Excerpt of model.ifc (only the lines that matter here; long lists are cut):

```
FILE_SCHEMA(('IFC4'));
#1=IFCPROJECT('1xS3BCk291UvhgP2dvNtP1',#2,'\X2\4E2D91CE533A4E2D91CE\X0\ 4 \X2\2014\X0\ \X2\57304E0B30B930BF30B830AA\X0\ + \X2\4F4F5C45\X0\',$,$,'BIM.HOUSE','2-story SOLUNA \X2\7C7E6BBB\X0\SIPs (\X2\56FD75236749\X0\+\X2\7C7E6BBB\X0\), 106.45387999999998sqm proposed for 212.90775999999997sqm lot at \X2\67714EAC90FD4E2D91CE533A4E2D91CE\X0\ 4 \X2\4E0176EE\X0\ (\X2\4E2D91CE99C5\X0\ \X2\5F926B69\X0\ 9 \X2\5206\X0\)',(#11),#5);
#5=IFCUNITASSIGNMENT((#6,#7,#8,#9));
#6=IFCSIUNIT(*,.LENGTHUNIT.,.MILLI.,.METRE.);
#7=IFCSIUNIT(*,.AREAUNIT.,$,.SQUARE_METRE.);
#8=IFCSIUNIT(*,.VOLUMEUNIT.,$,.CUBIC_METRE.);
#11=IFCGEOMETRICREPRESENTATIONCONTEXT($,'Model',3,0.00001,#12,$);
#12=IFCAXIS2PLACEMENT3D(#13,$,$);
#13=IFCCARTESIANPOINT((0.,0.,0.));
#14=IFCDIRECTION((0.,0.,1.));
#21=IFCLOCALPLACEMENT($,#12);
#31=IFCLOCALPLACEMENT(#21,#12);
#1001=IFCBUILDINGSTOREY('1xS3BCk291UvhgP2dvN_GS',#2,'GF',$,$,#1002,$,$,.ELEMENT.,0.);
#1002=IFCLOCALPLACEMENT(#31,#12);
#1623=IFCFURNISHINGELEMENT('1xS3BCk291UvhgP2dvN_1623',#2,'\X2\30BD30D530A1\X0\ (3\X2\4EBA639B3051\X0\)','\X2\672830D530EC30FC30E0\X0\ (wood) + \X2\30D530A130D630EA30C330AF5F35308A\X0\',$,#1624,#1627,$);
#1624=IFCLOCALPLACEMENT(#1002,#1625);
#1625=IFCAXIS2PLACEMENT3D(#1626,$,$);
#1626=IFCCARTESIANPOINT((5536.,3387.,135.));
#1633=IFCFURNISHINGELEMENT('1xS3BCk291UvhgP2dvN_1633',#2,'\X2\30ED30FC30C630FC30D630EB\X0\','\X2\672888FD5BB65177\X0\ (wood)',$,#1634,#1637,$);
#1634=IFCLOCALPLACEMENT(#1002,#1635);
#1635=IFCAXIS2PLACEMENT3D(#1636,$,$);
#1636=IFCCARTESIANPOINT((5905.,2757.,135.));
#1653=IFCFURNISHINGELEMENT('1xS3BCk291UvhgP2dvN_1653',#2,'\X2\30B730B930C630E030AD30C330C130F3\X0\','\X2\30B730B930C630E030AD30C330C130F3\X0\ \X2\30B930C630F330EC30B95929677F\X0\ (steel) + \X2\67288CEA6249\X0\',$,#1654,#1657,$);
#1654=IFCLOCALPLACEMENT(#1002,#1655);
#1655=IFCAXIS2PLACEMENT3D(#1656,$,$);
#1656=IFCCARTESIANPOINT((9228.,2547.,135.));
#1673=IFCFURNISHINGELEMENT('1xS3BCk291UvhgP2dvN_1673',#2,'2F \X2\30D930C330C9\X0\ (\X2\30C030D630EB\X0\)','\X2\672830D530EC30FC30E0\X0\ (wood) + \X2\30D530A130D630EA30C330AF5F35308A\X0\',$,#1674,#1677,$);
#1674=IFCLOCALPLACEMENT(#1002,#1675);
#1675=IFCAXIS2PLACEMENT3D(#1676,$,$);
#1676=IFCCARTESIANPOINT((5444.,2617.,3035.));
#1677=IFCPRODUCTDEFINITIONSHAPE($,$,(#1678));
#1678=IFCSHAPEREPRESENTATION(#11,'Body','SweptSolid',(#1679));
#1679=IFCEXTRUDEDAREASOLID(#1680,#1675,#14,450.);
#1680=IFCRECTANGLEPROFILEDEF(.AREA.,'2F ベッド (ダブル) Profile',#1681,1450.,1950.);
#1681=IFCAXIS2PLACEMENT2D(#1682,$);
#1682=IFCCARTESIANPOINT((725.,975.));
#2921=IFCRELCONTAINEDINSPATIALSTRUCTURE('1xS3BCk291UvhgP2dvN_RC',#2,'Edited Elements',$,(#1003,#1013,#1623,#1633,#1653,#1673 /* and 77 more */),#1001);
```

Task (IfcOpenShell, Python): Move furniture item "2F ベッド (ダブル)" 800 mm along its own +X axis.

```python
import ifcopenshell
import ifcopenshell.api.geometry
import ifcopenshell.util.placement

model = ifcopenshell.open("model.ifc")

item = model.by_guid("1xS3BCk291UvhgP2dvN_1673")
matrix = ifcopenshell.util.placement.get_local_placement(item.ObjectPlacement)
matrix[:3, 3] += matrix[:3, 0] * 800.0
ifcopenshell.api.geometry.edit_object_placement(model, product=item, matrix=matrix, is_si=False)

print(ifcopenshell.util.placement.get_local_placement(item.ObjectPlacement).round(3) + 0.0)

model.write("model_edited.ifc")
```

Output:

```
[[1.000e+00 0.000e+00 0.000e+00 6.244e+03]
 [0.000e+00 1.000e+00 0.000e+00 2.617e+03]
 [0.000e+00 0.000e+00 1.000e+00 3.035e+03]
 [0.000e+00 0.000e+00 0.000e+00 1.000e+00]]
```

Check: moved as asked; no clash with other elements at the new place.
